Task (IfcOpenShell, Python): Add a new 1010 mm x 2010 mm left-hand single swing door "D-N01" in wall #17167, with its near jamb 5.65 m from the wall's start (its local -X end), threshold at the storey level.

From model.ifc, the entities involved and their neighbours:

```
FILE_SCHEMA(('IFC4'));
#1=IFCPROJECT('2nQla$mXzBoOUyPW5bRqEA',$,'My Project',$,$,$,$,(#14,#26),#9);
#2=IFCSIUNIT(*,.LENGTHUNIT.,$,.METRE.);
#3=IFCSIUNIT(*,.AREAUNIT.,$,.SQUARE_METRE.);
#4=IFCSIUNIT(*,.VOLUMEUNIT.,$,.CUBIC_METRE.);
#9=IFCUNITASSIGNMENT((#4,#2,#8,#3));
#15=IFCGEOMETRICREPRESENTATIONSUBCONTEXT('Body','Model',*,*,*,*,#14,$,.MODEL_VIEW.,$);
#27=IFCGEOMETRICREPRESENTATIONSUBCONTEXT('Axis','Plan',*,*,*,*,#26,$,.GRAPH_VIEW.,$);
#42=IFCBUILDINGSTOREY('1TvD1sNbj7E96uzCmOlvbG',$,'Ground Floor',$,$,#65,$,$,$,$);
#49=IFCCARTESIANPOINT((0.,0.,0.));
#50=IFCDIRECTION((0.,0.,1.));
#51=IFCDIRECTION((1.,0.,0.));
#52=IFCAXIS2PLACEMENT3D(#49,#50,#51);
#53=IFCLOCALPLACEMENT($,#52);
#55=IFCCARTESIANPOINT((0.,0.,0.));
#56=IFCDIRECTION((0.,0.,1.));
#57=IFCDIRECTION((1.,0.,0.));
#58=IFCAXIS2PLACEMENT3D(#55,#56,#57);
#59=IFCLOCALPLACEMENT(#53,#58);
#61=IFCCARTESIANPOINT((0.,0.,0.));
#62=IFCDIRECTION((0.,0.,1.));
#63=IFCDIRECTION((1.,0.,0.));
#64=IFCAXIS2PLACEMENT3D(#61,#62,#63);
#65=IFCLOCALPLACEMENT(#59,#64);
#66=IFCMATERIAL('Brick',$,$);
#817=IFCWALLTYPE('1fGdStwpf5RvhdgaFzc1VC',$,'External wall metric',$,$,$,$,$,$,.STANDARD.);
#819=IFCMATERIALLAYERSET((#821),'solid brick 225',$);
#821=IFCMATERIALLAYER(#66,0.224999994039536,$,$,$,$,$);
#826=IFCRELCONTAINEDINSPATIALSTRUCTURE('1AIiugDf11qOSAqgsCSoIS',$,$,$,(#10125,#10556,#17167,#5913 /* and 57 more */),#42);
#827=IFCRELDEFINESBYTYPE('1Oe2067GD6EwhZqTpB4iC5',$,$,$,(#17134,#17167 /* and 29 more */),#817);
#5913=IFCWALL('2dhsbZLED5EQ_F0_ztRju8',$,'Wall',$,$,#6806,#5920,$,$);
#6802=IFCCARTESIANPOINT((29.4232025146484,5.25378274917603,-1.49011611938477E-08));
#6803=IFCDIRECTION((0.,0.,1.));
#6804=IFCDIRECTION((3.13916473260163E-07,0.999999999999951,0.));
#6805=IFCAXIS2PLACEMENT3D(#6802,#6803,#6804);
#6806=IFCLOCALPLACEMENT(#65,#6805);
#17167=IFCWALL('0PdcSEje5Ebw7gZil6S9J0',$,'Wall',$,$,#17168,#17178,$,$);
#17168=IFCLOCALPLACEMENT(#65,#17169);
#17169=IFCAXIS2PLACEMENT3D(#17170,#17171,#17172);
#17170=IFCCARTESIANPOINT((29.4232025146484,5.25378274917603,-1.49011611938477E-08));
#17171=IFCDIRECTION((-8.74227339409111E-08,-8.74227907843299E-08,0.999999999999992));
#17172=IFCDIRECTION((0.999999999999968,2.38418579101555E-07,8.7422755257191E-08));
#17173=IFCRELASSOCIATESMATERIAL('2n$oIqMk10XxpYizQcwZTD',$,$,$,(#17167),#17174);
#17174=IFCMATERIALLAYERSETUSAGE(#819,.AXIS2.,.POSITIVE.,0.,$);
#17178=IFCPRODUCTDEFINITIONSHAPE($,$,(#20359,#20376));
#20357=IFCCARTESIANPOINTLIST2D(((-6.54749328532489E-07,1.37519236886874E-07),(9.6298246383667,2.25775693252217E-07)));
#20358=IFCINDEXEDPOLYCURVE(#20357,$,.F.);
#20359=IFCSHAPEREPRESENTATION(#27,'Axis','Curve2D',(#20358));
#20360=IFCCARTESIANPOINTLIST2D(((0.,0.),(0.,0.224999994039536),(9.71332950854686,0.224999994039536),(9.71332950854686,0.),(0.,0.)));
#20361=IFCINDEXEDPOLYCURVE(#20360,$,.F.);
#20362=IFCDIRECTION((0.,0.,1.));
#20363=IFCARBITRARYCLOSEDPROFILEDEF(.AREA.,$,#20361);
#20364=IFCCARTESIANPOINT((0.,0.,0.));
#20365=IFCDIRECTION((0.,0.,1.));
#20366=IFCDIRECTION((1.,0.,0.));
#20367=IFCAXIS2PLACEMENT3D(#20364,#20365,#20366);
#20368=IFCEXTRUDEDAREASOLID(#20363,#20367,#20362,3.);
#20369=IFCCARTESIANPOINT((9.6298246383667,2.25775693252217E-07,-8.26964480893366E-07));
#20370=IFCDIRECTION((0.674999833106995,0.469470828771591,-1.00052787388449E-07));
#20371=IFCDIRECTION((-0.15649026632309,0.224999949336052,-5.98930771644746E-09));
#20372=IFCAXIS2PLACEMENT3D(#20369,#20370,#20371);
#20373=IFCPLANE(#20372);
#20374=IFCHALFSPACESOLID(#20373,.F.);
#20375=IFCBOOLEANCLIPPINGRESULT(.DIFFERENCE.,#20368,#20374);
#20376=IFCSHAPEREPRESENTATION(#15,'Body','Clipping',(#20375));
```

```python
import numpy as np
import ifcopenshell
import ifcopenshell.api.feature
import ifcopenshell.api.geometry
import ifcopenshell.api.root
import ifcopenshell.api.spatial
import ifcopenshell.geom
import ifcopenshell.util.element
import ifcopenshell.util.placement
import ifcopenshell.util.representation
import ifcopenshell.util.shape
import ifcopenshell.util.unit

model = ifcopenshell.open("model.ifc")
unit_scale = ifcopenshell.util.unit.calculate_unit_scale(model)
settings = ifcopenshell.geom.settings()


def volume(element):
    """Net volume in cubic metres, openings subtracted."""
    shape = ifcopenshell.geom.create_shape(settings, element)
    return ifcopenshell.util.shape.get_volume(shape.geometry)


wall = model.by_guid("0PdcSEje5Ebw7gZil6S9J0")
storey = ifcopenshell.util.element.get_container(wall, ifc_class="IfcBuildingStorey")
context = ifcopenshell.util.representation.get_context(model, "Model", "Body", "MODEL_VIEW")
before = volume(wall)

width, height, from_end, sill = 1.01, 2.01, 5.65, 0.0  # metres

# The wall runs along its own X axis, and the end named is its -X end.
wall_shape = ifcopenshell.geom.create_shape(settings, wall)
x, y, z = ifcopenshell.util.shape.get_vertices(wall_shape.geometry).T
start = x.min() + from_end
face, thickness = float(y.min()), float(y.max() - y.min())
wall_matrix = ifcopenshell.util.placement.get_local_placement(wall.ObjectPlacement)
level = ifcopenshell.util.placement.get_local_placement(storey.ObjectPlacement)[2, 3]


def in_wall(x, y):
    """Placement at x, y metres in the wall's axes, at sill height."""
    matrix = wall_matrix.copy()
    matrix[:, 3] = wall_matrix @ np.array([x / unit_scale, y / unit_scale, 0.0, 1.0])
    matrix[2, 3] = level + sill / unit_scale
    return matrix


# Opening: a box that overshoots both wall faces by 50 mm.
opening = ifcopenshell.api.root.create_entity(model, ifc_class="IfcOpeningElement", predefined_type="OPENING")
box = ifcopenshell.api.geometry.add_wall_representation(
    model, context=context, length=width, height=height, thickness=thickness + 0.1
)
ifcopenshell.api.geometry.assign_representation(model, product=opening, representation=box)
ifcopenshell.api.geometry.edit_object_placement(model, product=opening, matrix=in_wall(start, face - 0.05), is_si=False)
ifcopenshell.api.feature.add_feature(model, feature=opening, element=wall)

door = ifcopenshell.api.root.create_entity(model, ifc_class="IfcDoor", name="D-N01", predefined_type="DOOR")
door.OverallWidth, door.OverallHeight = width / unit_scale, height / unit_scale
door.OperationType = "SINGLE_SWING_LEFT"
body = ifcopenshell.api.geometry.add_door_representation(
    model,
    context=context,
    overall_width=door.OverallWidth,
    overall_height=door.OverallHeight,
    operation_type="SINGLE_SWING_LEFT",
    lining_properties={"LiningDepth": thickness / unit_scale, "ThresholdDepth": thickness / unit_scale},
)
ifcopenshell.api.geometry.assign_representation(model, product=door, representation=body)
ifcopenshell.api.spatial.assign_container(model, products=[door], relating_structure=storey)
ifcopenshell.api.feature.add_filling(model, opening=opening, element=door)

# The lining spans the wall, so the door starts at the wall face.
ifcopenshell.api.geometry.edit_object_placement(model, product=door, matrix=in_wall(start, face), is_si=False)

after = volume(wall)

print(f"wall volume {before:.3f} -> {after:.3f} m3")

model.write("model_edited.ifc")
```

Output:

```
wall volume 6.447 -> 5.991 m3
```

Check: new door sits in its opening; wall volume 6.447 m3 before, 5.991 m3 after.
